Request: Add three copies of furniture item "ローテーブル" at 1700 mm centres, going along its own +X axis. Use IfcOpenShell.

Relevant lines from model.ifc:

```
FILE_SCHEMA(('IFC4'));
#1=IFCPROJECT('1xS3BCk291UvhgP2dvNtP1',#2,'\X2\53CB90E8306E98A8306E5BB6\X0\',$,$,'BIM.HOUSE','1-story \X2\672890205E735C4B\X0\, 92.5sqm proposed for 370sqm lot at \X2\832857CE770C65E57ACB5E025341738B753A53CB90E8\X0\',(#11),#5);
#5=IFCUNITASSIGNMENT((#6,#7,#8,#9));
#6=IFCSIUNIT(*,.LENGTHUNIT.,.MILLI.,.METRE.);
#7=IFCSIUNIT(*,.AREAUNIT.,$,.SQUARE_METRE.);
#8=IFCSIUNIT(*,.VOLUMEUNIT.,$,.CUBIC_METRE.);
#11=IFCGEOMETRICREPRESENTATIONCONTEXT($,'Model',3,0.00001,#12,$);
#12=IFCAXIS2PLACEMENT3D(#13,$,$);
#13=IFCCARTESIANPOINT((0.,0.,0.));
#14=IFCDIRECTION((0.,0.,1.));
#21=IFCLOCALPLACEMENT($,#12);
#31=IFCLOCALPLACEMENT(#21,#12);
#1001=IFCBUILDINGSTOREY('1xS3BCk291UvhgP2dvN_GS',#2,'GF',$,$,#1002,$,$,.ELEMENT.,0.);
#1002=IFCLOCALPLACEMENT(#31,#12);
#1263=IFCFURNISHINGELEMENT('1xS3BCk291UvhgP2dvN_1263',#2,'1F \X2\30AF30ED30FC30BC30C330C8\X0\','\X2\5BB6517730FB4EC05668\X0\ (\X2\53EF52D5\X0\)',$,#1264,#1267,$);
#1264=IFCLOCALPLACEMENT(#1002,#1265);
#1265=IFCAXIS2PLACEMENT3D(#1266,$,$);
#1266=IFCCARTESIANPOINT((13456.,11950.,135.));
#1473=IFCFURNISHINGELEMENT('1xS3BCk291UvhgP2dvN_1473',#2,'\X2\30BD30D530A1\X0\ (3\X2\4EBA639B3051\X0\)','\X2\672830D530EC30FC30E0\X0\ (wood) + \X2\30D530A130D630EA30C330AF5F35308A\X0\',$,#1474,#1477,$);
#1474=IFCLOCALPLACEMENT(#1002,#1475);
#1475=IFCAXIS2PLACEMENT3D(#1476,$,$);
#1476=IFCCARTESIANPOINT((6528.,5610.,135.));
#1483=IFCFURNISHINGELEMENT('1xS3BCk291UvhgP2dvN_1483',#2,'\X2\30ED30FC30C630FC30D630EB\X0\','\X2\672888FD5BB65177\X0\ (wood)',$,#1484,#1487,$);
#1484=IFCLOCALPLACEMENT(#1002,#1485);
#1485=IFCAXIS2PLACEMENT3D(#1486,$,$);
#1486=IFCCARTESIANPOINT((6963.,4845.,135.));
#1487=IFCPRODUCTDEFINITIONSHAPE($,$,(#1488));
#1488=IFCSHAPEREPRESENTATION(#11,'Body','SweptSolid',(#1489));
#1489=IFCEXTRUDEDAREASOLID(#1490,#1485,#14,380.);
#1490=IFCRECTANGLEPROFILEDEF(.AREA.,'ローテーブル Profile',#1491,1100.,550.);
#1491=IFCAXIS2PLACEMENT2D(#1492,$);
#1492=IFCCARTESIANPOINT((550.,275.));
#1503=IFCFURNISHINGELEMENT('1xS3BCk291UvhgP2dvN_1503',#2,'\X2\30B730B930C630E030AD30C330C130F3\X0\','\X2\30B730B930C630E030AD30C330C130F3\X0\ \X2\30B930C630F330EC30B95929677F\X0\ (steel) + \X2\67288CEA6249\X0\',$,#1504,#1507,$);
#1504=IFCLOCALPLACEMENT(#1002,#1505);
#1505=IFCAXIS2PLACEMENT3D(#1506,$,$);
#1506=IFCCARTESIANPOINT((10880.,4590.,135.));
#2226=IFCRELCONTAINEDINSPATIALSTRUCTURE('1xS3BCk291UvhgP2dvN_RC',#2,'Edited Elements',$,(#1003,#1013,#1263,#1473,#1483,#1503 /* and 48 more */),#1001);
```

```python
import ifcopenshell
import ifcopenshell.api.geometry
import ifcopenshell.api.root
import ifcopenshell.util.element
import ifcopenshell.util.placement

model = ifcopenshell.open("model.ifc")


def reuse_history(source, copy):
    """copy_class also copies each property set's owner history, people and application; keep the originals."""
    for rel in copy.IsDefinedBy:
        if rel.is_a("IfcRelDefinesByProperties") and (history := rel.RelatingPropertyDefinition.OwnerHistory):
            rel.RelatingPropertyDefinition.OwnerHistory = source.OwnerHistory
            ifcopenshell.util.element.remove_deep2(model, history)


source = model.by_guid("1xS3BCk291UvhgP2dvN_1483")
base = ifcopenshell.util.placement.get_local_placement(source.ObjectPlacement)
step = base[:3, 0] * 1700.0

for i in range(1, 4):
    copy = ifcopenshell.api.root.copy_class(model, product=source)
    copy.Representation = ifcopenshell.util.element.copy_deep(
        model, source.Representation, exclude=["IfcGeometricRepresentationContext", "IfcRepresentationMap"]
    )
    reuse_history(source, copy)
    matrix = base.copy()
    matrix[:3, 3] += i * step
    print("added at", matrix[:3, 3].round(3) + 0.0)
    ifcopenshell.api.geometry.edit_object_placement(model, product=copy, matrix=matrix, is_si=False)

model.write("model_rev.ifc")
```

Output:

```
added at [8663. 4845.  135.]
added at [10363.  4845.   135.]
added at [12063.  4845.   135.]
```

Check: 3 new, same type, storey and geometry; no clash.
